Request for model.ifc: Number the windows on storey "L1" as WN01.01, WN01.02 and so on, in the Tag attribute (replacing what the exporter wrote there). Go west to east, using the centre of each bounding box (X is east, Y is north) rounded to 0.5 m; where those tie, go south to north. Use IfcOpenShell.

First a look at what the model holds.

```python
import ifcopenshell
import ifcopenshell.util.element
import ifcopenshell.util.placement

model = ifcopenshell.open("model.ifc")
print(model.schema)
storey = next(s for s in model.by_type("IfcBuildingStorey") if s.Name == "L1")
windows = [e for e in ifcopenshell.util.element.get_decomposition(storey) if e.is_a("IfcWindow")]
for e in sorted(windows, key=lambda e: e.id()):
    origin = ifcopenshell.util.placement.get_local_placement(e.ObjectPlacement)[:3, 3]
    print(e.id(), e.Tag, e.Name, origin.round(2) + 0.0, sep=" | ")
```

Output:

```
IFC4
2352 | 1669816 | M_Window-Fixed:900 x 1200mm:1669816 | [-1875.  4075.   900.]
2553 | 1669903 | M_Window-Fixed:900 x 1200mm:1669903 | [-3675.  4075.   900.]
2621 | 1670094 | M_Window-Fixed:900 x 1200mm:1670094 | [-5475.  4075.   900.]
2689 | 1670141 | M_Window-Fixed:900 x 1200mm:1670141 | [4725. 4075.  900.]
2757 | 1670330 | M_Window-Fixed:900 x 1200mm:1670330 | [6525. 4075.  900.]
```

```python
import ifcopenshell
import ifcopenshell.geom
import ifcopenshell.util.element
import ifcopenshell.util.shape

model = ifcopenshell.open("model.ifc")
settings = ifcopenshell.geom.settings()
settings.set("use-world-coords", True)


def centre(element):
    shape = ifcopenshell.geom.create_shape(settings, element)
    return ifcopenshell.util.shape.get_bbox_centroid(shape.geometry)


storey = next(s for s in model.by_type("IfcBuildingStorey") if s.Name == "L1")
windows = [e for e in ifcopenshell.util.element.get_decomposition(storey) if e.is_a("IfcWindow")]

# Insertion points can sit at a corner or the storey origin, so sort by the geometry (in metres).
centres = {e: centre(e) for e in windows}
windows.sort(key=lambda e: (round(centres[e][0] / 0.5), centres[e][1]))

for i, e in enumerate(windows, start=1):
    number = f"WN01.{i:02d}"
    e.Tag = number
    print(e.id(), number)

model.write("model_v2.ifc")
```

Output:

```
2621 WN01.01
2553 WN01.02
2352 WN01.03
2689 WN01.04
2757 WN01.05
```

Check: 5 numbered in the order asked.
